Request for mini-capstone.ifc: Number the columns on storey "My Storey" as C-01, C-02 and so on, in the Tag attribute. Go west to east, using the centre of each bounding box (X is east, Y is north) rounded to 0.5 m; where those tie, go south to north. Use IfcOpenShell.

First a look at what the model holds.

```python
import ifcopenshell
import ifcopenshell.util.element
import ifcopenshell.util.placement

model = ifcopenshell.open("mini-capstone.ifc")
print(model.schema)
storey = next(s for s in model.by_type("IfcBuildingStorey") if s.Name == "My Storey")
columns = [e for e in ifcopenshell.util.element.get_decomposition(storey) if e.is_a("IfcColumn")]
for e in sorted(columns, key=lambda e: e.id()):
    origin = ifcopenshell.util.placement.get_local_placement(e.ObjectPlacement)[:3, 3]
    print(e.id(), e.Tag, e.Name, origin.round(2) + 0.0, sep=" | ")
```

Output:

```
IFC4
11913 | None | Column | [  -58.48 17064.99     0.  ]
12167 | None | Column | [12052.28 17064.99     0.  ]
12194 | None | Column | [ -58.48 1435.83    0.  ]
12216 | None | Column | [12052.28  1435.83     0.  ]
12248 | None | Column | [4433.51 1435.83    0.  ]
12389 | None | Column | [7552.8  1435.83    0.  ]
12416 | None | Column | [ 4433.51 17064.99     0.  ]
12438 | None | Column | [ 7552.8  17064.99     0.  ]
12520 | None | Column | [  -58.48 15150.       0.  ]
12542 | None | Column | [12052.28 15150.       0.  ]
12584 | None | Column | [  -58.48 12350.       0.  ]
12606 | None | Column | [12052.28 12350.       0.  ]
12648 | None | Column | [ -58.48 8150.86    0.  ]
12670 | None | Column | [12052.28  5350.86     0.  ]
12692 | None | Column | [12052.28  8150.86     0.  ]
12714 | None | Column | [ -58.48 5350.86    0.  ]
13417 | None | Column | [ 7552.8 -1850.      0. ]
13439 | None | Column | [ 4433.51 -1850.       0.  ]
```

```python
import ifcopenshell
import ifcopenshell.geom
import ifcopenshell.util.element
import ifcopenshell.util.shape

model = ifcopenshell.open("mini-capstone.ifc")
settings = ifcopenshell.geom.settings()
settings.set("use-world-coords", True)


def centre(element):
    shape = ifcopenshell.geom.create_shape(settings, element)
    return ifcopenshell.util.shape.get_bbox_centroid(shape.geometry)


storey = next(s for s in model.by_type("IfcBuildingStorey") if s.Name == "My Storey")
columns = [e for e in ifcopenshell.util.element.get_decomposition(storey) if e.is_a("IfcColumn")]

# Insertion points can sit at a corner or the storey origin, so sort by the geometry (in metres).
centres = {e: centre(e) for e in columns}
columns.sort(key=lambda e: (round(centres[e][0] / 0.5), centres[e][1]))

for i, e in enumerate(columns, start=1):
    number = f"C-{i:02d}"
    e.Tag = number
    print(e.id(), number)

model.write("mini-capstone_updated.ifc")
```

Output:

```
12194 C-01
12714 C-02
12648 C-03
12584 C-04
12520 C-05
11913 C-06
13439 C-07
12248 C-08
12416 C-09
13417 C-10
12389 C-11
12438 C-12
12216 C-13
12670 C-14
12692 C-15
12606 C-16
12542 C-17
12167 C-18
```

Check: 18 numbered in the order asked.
